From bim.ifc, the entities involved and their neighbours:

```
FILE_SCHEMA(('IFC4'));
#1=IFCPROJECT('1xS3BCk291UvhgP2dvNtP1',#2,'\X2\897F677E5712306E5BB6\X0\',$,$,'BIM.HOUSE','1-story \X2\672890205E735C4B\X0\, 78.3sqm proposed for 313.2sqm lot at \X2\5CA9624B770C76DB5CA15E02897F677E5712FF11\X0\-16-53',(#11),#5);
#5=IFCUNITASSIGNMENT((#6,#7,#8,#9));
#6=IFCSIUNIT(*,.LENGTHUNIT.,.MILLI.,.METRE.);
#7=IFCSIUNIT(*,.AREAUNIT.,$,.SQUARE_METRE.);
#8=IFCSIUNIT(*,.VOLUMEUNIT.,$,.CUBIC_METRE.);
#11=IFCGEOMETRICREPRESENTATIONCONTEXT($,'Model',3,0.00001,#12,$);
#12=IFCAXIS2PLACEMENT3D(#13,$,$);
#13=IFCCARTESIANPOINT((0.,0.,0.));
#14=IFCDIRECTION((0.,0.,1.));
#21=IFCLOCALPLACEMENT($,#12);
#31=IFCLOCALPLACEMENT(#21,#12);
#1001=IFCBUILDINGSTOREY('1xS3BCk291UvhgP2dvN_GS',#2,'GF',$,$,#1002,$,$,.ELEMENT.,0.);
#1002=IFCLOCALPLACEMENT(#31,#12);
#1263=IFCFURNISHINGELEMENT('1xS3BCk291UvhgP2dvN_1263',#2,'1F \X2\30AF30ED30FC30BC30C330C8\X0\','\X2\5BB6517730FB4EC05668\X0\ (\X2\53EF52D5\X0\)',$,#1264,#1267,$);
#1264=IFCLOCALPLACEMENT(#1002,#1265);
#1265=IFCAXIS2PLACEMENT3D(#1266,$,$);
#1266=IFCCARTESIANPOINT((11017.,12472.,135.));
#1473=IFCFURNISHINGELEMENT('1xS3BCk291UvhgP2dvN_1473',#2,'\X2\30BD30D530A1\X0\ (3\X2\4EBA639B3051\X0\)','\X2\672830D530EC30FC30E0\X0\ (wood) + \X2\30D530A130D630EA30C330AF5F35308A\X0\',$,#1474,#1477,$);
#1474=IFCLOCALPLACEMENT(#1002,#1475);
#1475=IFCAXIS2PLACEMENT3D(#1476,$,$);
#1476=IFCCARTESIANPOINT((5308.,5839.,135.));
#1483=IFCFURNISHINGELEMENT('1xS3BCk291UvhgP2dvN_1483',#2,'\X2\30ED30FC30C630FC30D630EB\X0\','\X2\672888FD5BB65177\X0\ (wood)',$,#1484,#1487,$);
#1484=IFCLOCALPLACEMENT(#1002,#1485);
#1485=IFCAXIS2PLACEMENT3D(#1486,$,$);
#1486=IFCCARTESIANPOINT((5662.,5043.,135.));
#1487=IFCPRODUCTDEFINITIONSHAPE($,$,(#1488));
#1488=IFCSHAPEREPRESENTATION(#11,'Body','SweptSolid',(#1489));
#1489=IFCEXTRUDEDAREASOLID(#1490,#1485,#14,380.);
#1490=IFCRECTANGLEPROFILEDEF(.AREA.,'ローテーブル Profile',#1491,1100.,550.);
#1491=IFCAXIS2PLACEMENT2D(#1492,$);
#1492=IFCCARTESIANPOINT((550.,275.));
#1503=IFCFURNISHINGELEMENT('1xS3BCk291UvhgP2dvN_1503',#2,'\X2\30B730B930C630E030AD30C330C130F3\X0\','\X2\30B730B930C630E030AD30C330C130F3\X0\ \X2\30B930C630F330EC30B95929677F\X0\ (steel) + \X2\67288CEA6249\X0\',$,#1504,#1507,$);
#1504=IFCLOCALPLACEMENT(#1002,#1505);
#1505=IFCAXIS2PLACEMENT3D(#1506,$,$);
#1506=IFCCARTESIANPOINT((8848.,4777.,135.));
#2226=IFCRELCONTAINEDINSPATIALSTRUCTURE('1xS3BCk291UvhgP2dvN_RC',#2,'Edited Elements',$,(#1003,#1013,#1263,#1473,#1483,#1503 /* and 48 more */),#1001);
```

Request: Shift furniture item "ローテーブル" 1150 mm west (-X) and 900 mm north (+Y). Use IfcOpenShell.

```python
import ifcopenshell
import ifcopenshell.api.geometry
import ifcopenshell.util.placement
import ifcopenshell.util.unit

model = ifcopenshell.open("bim.ifc")
unit_scale = ifcopenshell.util.unit.calculate_unit_scale(model)

item = model.by_guid("1xS3BCk291UvhgP2dvN_1483")
matrix = ifcopenshell.util.placement.get_local_placement(item.ObjectPlacement)
matrix[0, 3] -= 1.15 / unit_scale
matrix[1, 3] += 0.9 / unit_scale
ifcopenshell.api.geometry.edit_object_placement(model, product=item, matrix=matrix, is_si=False)

print(ifcopenshell.util.placement.get_local_placement(item.ObjectPlacement).round(3) + 0.0)

model.write("bim-out.ifc")
```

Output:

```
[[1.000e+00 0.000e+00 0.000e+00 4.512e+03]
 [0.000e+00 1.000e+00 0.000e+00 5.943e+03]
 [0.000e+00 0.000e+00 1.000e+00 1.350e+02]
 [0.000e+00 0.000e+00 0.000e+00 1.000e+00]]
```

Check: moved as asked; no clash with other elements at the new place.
